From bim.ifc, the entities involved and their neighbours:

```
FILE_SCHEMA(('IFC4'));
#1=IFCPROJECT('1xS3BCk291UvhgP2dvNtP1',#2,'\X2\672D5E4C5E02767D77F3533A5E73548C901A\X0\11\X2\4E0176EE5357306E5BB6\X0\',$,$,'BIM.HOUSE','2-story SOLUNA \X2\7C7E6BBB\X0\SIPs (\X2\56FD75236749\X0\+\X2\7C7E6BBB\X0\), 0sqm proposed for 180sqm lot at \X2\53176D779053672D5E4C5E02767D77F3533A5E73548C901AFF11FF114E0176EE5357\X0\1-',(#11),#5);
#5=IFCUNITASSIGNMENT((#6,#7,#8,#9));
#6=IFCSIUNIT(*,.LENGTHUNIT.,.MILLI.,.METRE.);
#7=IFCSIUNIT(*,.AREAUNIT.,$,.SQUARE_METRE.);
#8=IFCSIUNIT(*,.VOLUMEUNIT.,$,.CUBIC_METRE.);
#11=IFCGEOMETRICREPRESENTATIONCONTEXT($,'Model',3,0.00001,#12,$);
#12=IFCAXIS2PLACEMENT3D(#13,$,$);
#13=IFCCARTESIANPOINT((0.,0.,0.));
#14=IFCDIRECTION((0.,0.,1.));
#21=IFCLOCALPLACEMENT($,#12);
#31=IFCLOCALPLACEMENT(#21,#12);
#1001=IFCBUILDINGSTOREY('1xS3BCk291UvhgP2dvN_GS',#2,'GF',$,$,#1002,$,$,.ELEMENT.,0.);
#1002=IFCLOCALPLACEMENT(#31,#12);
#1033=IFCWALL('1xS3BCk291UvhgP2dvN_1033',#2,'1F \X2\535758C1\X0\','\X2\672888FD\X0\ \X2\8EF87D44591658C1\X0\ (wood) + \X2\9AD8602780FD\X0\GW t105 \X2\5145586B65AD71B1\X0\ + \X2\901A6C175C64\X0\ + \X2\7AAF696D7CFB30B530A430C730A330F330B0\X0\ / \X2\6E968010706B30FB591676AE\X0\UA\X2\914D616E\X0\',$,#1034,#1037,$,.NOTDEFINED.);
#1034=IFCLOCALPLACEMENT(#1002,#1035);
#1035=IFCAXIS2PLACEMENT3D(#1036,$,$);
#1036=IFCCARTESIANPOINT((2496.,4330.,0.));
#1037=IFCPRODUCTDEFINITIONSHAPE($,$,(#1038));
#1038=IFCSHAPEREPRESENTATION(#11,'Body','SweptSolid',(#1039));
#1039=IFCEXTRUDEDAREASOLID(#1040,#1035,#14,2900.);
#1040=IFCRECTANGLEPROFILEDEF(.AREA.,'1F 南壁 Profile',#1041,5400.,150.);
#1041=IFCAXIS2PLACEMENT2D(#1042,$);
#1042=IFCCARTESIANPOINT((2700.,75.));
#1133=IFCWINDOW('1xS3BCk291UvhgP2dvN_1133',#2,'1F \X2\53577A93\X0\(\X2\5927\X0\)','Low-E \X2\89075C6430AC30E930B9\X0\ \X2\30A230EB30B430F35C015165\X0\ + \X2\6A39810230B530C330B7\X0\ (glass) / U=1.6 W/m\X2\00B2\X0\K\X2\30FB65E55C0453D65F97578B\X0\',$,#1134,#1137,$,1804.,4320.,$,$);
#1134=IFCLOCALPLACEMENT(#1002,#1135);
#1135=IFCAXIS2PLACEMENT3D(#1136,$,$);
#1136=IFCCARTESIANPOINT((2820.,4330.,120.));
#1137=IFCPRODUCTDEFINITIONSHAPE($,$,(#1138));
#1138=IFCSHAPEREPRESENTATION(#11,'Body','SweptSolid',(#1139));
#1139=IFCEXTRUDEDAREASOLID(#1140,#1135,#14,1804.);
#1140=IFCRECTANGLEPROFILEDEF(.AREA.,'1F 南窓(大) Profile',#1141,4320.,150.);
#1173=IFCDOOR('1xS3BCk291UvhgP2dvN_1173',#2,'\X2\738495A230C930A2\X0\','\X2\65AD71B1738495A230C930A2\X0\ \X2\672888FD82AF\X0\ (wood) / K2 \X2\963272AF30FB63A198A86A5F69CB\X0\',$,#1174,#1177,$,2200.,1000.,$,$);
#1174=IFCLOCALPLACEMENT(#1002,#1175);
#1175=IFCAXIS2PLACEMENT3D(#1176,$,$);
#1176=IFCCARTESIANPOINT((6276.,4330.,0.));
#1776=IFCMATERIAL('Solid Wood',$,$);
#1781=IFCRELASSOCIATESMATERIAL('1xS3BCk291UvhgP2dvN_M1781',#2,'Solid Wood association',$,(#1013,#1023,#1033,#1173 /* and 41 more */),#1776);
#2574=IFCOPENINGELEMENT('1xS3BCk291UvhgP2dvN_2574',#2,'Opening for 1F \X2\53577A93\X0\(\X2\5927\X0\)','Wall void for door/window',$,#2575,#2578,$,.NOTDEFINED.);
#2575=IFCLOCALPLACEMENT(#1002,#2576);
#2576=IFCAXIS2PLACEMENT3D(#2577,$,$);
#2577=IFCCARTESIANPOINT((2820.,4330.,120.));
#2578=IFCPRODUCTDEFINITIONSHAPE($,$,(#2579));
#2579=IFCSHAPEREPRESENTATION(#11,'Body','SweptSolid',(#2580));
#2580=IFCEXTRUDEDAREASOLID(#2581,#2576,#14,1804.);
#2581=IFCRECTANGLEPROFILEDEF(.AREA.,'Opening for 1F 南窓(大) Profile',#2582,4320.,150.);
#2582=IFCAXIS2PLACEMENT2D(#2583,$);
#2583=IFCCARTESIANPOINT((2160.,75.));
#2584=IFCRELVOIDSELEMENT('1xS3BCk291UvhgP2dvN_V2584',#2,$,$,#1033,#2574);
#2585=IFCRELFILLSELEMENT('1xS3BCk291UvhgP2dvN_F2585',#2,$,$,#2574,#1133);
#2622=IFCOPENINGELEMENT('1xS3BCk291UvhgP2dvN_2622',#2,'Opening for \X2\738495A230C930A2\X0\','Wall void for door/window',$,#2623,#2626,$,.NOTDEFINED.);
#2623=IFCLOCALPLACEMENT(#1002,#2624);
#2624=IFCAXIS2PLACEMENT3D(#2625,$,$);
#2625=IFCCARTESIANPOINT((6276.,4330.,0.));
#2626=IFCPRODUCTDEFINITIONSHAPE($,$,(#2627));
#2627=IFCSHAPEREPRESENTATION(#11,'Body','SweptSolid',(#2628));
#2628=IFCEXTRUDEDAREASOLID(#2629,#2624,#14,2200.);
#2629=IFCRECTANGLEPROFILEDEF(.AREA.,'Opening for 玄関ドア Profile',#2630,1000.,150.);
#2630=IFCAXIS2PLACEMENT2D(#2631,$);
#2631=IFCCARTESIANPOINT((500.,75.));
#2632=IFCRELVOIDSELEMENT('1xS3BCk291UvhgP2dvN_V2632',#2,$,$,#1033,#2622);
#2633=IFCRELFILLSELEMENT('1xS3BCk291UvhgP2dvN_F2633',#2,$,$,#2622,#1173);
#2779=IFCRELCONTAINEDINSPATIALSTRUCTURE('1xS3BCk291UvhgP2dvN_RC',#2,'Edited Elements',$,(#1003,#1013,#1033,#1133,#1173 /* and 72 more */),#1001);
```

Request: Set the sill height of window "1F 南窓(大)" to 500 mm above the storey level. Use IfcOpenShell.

```python
import numpy as np
import ifcopenshell
import ifcopenshell.api.geometry
import ifcopenshell.geom
import ifcopenshell.util.element
import ifcopenshell.util.placement
import ifcopenshell.util.shape
import ifcopenshell.util.unit

model = ifcopenshell.open("bim.ifc")
unit_scale = ifcopenshell.util.unit.calculate_unit_scale(model)

window = model.by_id(1133)
opening = window.FillsVoids[0].RelatingOpeningElement
storey = ifcopenshell.util.element.get_container(window, ifc_class="IfcBuildingStorey")
level = ifcopenshell.util.placement.get_local_placement(storey.ObjectPlacement)[2, 3]

# The opening's origin need not be at the sill, so measure its lowest point.
shape = ifcopenshell.geom.create_shape(ifcopenshell.geom.settings(), opening)
bottom = ifcopenshell.util.shape.get_shape_bottom_elevation(shape, shape.geometry) / unit_scale
dz = level + 500.0 - bottom

shift = np.array([0.0, 0.0, dz])
# The window is not placed relative to its opening, so move both.
for product in (opening, window):
    matrix = ifcopenshell.util.placement.get_local_placement(product.ObjectPlacement)
    matrix[:3, 3] += shift
    ifcopenshell.api.geometry.edit_object_placement(model, product=product, matrix=matrix, is_si=False)

print(f"moved by {dz * unit_scale:+.3f} m")

model.write("bim_v2.ifc")
```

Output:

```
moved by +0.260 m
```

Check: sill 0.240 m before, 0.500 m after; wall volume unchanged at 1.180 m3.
